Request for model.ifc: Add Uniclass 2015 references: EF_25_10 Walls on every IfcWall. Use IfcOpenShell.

First a look at what the model holds.

```python
import ifcopenshell

model = ifcopenshell.open("model.ifc")
print(model.schema)
print("classifications:", [c.Name for c in model.by_type("IfcClassification")])
for ifc_class in ("IfcDoor", "IfcRoof", "IfcStair", "IfcWall", "IfcWindow"):
    print(ifc_class, len(model.by_type(ifc_class)))
```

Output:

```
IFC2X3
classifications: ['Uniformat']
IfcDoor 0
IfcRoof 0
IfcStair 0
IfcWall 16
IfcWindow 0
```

```python
import ifcopenshell
import ifcopenshell.api.classification

model = ifcopenshell.open("model.ifc")

# IFC2X3 requires Source and Edition and has no link from the project to the system.
system = model.create_entity("IfcClassification", Source="NBS", Edition="2015", Name="Uniclass 2015")

codes = {
    "IfcWall": ("EF_25_10", "Walls"),
}
for ifc_class, (code, name) in codes.items():
    products = model.by_type(ifc_class)
    ifcopenshell.api.classification.add_reference(
        model, products=products, classification=system, identification=code, name=name
    )
    print(code, len(products))

model.write("model_v2.ifc")
```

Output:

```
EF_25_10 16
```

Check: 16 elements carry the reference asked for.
